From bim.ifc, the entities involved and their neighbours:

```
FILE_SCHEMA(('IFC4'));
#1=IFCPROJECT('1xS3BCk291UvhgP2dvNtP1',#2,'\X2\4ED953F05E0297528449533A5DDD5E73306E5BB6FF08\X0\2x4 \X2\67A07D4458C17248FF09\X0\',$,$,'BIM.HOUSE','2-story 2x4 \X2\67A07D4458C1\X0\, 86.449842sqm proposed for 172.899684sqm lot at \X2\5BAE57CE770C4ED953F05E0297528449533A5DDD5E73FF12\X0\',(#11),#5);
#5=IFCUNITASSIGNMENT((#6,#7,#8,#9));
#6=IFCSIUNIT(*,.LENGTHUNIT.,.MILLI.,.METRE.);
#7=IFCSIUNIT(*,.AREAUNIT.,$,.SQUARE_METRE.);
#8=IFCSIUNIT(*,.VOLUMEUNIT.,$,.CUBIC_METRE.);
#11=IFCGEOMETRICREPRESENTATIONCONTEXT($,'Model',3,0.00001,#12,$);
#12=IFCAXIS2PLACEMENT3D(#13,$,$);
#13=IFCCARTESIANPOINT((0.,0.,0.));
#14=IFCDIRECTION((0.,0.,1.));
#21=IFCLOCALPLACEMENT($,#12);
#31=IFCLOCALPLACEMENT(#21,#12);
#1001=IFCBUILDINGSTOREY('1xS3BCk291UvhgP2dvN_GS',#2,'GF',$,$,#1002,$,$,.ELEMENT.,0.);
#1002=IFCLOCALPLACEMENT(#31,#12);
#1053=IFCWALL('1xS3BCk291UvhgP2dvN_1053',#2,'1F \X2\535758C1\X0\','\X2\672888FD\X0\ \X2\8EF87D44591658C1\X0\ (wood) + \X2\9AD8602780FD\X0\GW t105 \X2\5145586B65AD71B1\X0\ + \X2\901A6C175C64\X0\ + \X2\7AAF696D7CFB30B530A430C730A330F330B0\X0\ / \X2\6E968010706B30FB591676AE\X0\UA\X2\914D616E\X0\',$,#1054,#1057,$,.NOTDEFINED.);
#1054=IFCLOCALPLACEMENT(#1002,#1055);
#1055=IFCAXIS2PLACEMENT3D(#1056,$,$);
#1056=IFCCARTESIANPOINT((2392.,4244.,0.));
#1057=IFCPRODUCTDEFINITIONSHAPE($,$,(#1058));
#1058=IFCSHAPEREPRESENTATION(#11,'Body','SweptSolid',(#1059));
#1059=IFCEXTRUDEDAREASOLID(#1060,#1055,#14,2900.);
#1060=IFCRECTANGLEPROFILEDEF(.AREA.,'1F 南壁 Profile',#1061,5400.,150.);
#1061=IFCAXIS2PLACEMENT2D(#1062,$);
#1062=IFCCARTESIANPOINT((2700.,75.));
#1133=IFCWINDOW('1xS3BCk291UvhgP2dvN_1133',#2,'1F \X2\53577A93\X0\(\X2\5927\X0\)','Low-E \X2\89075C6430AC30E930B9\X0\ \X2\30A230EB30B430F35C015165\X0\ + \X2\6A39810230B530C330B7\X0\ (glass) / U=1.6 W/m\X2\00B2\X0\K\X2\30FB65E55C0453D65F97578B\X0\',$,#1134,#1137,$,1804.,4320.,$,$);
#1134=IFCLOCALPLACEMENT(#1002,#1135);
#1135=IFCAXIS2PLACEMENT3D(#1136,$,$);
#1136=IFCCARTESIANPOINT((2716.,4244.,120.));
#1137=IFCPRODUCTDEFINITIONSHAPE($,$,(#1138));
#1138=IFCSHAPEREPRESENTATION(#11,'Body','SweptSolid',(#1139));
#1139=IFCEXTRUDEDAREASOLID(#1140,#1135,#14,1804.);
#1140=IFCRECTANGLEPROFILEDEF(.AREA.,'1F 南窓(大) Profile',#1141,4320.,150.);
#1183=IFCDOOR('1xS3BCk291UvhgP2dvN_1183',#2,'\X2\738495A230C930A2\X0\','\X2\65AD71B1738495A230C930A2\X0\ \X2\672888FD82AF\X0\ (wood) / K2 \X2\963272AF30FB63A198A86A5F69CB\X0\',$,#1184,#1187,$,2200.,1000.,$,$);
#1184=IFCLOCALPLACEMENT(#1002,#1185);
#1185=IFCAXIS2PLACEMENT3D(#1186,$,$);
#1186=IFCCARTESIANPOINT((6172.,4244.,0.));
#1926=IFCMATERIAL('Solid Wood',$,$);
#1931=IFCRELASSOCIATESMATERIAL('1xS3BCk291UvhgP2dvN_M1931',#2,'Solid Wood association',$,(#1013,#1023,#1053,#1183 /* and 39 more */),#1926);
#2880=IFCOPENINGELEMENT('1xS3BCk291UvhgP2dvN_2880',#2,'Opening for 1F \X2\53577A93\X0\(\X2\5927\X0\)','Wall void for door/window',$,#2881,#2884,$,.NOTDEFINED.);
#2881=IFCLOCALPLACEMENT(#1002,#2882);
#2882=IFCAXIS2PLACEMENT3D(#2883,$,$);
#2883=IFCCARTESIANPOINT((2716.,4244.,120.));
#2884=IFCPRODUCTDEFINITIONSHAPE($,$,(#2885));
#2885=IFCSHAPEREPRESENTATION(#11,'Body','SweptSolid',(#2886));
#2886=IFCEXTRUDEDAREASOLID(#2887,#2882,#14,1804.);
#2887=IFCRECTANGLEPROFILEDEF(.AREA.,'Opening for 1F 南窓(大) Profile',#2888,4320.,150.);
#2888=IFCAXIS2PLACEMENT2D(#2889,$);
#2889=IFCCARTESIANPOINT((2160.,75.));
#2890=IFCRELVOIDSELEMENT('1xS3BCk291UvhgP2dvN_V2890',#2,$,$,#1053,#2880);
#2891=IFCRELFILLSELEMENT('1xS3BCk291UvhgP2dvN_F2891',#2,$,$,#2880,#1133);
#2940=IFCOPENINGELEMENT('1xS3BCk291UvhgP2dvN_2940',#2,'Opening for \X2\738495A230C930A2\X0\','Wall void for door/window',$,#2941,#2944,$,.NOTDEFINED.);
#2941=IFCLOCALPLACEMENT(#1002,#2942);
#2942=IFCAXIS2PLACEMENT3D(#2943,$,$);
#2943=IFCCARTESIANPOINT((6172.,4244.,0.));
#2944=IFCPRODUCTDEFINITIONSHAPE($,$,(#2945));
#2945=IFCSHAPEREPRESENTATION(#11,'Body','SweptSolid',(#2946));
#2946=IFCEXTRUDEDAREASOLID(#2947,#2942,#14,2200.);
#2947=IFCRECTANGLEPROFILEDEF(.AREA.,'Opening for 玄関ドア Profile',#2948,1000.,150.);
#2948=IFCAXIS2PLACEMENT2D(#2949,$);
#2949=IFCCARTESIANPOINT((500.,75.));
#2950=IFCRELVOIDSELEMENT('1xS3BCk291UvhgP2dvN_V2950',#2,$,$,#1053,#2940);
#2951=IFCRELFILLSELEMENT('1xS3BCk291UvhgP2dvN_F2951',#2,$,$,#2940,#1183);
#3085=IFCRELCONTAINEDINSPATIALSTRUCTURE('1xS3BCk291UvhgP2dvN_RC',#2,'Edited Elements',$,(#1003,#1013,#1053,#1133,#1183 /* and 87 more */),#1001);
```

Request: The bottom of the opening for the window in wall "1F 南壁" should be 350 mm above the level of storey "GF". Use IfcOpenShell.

```python
import numpy as np
import ifcopenshell
import ifcopenshell.api.geometry
import ifcopenshell.geom
import ifcopenshell.util.element
import ifcopenshell.util.placement
import ifcopenshell.util.shape
import ifcopenshell.util.unit

model = ifcopenshell.open("bim.ifc")
unit_scale = ifcopenshell.util.unit.calculate_unit_scale(model)

window = model.by_id(1133)
opening = window.FillsVoids[0].RelatingOpeningElement
storey = ifcopenshell.util.element.get_container(window, ifc_class="IfcBuildingStorey")
level = ifcopenshell.util.placement.get_local_placement(storey.ObjectPlacement)[2, 3]

# The opening's origin need not be at the sill, so measure its lowest point.
shape = ifcopenshell.geom.create_shape(ifcopenshell.geom.settings(), opening)
bottom = ifcopenshell.util.shape.get_shape_bottom_elevation(shape, shape.geometry) / unit_scale
dz = level + 350.0 - bottom

shift = np.array([0.0, 0.0, dz])
# The window is not placed relative to its opening, so move both.
for product in (opening, window):
    matrix = ifcopenshell.util.placement.get_local_placement(product.ObjectPlacement)
    matrix[:3, 3] += shift
    ifcopenshell.api.geometry.edit_object_placement(model, product=product, matrix=matrix, is_si=False)

print(f"moved by {dz * unit_scale:+.3f} m")

model.write("bim_v2.ifc")
```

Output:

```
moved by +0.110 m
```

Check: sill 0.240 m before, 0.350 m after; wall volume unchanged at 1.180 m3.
